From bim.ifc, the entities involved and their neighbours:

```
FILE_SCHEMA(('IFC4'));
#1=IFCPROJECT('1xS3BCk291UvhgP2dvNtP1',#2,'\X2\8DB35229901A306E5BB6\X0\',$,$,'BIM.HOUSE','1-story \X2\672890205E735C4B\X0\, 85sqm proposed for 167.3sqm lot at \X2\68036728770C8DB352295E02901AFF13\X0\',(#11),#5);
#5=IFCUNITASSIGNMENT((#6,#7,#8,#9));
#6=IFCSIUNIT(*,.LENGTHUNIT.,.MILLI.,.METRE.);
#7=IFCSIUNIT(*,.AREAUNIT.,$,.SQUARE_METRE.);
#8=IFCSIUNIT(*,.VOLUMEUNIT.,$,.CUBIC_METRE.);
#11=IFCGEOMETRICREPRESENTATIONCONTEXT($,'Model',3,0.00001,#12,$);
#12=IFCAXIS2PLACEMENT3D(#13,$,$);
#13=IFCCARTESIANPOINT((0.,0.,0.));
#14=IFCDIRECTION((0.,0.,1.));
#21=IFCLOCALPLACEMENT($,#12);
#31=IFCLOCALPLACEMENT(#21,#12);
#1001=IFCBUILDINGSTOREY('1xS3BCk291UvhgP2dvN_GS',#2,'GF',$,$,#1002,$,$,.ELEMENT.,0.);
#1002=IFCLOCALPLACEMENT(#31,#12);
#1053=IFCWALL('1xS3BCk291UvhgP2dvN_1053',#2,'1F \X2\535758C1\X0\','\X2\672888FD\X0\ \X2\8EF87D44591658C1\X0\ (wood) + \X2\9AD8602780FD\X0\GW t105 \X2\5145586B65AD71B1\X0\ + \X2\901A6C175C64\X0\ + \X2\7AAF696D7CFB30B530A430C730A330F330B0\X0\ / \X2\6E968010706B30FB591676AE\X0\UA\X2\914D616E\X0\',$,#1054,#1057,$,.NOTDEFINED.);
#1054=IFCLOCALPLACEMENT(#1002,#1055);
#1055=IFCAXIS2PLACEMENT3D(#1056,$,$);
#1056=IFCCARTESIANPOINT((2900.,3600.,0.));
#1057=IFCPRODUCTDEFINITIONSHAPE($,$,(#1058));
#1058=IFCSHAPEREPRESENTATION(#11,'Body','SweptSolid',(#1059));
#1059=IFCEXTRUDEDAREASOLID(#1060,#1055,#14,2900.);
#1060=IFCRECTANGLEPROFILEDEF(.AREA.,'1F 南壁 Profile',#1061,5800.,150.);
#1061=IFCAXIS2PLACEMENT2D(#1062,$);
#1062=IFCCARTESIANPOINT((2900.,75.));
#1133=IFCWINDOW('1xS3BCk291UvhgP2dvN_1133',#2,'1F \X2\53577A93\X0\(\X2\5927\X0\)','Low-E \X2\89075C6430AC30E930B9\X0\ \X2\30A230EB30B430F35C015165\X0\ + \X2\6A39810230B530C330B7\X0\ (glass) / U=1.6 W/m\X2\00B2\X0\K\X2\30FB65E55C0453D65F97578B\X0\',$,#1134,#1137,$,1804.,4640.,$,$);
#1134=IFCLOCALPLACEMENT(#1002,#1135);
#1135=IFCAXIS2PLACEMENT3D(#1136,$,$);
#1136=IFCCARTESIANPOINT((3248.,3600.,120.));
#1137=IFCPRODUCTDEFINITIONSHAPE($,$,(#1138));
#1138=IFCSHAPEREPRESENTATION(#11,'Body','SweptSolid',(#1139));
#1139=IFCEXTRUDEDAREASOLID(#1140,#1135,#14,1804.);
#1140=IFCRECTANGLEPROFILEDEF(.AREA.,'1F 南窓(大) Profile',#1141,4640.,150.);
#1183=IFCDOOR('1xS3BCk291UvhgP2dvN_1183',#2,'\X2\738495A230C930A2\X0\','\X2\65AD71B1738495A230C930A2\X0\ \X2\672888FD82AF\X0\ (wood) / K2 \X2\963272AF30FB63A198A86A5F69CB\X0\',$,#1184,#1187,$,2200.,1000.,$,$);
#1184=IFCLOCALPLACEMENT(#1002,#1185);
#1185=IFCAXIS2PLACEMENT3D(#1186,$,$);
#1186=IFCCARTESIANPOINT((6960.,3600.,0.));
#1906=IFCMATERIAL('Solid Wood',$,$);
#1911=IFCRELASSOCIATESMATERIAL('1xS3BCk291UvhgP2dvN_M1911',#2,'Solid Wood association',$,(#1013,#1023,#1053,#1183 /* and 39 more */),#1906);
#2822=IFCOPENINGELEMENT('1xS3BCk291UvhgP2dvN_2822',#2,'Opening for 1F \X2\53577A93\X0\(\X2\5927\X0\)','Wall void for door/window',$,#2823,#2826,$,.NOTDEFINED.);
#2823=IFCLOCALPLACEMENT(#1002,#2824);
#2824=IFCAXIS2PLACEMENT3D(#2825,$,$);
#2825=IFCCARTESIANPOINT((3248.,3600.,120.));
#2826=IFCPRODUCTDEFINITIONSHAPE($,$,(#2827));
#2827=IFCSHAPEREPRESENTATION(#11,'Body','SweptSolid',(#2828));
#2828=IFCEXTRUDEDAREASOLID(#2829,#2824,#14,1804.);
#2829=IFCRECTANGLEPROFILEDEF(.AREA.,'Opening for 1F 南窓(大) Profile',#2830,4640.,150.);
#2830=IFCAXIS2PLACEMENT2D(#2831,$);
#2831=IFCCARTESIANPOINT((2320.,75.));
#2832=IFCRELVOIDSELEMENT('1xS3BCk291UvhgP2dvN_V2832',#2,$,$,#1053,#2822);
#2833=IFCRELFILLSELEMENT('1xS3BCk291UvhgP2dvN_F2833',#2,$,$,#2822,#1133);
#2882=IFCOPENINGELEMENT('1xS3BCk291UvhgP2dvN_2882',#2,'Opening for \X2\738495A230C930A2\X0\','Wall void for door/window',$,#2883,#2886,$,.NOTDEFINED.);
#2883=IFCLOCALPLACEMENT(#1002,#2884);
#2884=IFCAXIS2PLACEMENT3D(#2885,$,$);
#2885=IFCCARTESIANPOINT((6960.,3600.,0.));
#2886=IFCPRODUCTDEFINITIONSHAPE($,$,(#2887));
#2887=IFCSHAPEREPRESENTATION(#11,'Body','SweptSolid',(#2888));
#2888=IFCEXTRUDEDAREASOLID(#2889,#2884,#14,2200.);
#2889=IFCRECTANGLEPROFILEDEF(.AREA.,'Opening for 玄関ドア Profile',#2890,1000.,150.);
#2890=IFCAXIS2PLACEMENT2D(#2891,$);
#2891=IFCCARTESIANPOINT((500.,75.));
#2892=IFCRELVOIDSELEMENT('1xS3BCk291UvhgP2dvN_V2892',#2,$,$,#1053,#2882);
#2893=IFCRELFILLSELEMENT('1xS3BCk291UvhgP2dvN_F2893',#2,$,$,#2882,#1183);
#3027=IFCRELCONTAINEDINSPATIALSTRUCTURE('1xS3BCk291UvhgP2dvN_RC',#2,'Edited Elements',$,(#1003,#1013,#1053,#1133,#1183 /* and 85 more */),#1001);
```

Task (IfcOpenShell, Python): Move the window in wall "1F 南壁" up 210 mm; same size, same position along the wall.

```python
import numpy as np
import ifcopenshell
import ifcopenshell.api.geometry
import ifcopenshell.util.placement
import ifcopenshell.util.unit

model = ifcopenshell.open("bim.ifc")
unit_scale = ifcopenshell.util.unit.calculate_unit_scale(model)

window = model.by_guid("1xS3BCk291UvhgP2dvN_1133")
opening = window.FillsVoids[0].RelatingOpeningElement
dz = 0.21 / unit_scale

shift = np.array([0.0, 0.0, dz])
# The window is not placed relative to its opening, so move both.
for product in (opening, window):
    matrix = ifcopenshell.util.placement.get_local_placement(product.ObjectPlacement)
    matrix[:3, 3] += shift
    ifcopenshell.api.geometry.edit_object_placement(model, product=product, matrix=matrix, is_si=False)

print(f"moved by {dz * unit_scale:+.3f} m")

model.write("bim-out.ifc")
```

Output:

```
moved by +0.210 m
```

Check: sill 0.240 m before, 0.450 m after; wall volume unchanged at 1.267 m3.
